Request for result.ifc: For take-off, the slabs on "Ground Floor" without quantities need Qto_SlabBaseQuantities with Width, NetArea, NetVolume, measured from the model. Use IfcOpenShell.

First a look at what the model holds.

```python
import ifcopenshell
import ifcopenshell.util.element
import ifcopenshell.util.unit

model = ifcopenshell.open("result.ifc")
print(model.schema)
for unit_type in ("LENGTHUNIT", "AREAUNIT", "VOLUMEUNIT"):
    print(unit_type, ifcopenshell.util.unit.calculate_unit_scale(model, unit_type))
storey = next(s for s in model.by_type("IfcBuildingStorey") if s.Name == "Ground Floor")
slabs = [e for e in ifcopenshell.util.element.get_decomposition(storey) if e.is_a("IfcSlab")]
for e in sorted(slabs, key=lambda e: e.id()):
    print(e.id(), e.is_a(), e.Name, list(ifcopenshell.util.element.get_psets(e, qtos_only=True)), sep=" | ")
```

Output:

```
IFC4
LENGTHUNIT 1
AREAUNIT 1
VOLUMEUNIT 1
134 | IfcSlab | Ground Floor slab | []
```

```python
import ifcopenshell
import ifcopenshell.api.pset
import ifcopenshell.geom
import ifcopenshell.util.element
import ifcopenshell.util.shape
import ifcopenshell.util.unit

model = ifcopenshell.open("result.ifc")
unit_scale = ifcopenshell.util.unit.calculate_unit_scale(model)
area_scale = ifcopenshell.util.unit.calculate_unit_scale(model, "AREAUNIT")
volume_scale = ifcopenshell.util.unit.calculate_unit_scale(model, "VOLUMEUNIT")
settings = ifcopenshell.geom.settings()

storey = next(s for s in model.by_type("IfcBuildingStorey") if s.Name == "Ground Floor")
slabs = [e for e in ifcopenshell.util.element.get_decomposition(storey) if e.is_a("IfcSlab")]

for e in sorted(slabs, key=lambda e: e.id()):
    if ifcopenshell.util.element.get_psets(e, qtos_only=True, should_inherit=False):
        continue
    # Geometry comes back in metres, in the element's own axes.
    shape = ifcopenshell.geom.create_shape(settings, e)
    values = {
        "Width": ifcopenshell.util.shape.get_z(shape.geometry) / unit_scale,
        "NetArea": ifcopenshell.util.shape.get_footprint_area(shape.geometry) / area_scale,
        "NetVolume": ifcopenshell.util.shape.get_volume(shape.geometry) / volume_scale,
    }
    qto = ifcopenshell.api.pset.add_qto(model, product=e, name="Qto_SlabBaseQuantities")
    ifcopenshell.api.pset.edit_qto(model, qto=qto, properties=values)
    print(e.id(), {k: round(v, 3) for k, v in values.items()})

model.write("result_v2.ifc")
```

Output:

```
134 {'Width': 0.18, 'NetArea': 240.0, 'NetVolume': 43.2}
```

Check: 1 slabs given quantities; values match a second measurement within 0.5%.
